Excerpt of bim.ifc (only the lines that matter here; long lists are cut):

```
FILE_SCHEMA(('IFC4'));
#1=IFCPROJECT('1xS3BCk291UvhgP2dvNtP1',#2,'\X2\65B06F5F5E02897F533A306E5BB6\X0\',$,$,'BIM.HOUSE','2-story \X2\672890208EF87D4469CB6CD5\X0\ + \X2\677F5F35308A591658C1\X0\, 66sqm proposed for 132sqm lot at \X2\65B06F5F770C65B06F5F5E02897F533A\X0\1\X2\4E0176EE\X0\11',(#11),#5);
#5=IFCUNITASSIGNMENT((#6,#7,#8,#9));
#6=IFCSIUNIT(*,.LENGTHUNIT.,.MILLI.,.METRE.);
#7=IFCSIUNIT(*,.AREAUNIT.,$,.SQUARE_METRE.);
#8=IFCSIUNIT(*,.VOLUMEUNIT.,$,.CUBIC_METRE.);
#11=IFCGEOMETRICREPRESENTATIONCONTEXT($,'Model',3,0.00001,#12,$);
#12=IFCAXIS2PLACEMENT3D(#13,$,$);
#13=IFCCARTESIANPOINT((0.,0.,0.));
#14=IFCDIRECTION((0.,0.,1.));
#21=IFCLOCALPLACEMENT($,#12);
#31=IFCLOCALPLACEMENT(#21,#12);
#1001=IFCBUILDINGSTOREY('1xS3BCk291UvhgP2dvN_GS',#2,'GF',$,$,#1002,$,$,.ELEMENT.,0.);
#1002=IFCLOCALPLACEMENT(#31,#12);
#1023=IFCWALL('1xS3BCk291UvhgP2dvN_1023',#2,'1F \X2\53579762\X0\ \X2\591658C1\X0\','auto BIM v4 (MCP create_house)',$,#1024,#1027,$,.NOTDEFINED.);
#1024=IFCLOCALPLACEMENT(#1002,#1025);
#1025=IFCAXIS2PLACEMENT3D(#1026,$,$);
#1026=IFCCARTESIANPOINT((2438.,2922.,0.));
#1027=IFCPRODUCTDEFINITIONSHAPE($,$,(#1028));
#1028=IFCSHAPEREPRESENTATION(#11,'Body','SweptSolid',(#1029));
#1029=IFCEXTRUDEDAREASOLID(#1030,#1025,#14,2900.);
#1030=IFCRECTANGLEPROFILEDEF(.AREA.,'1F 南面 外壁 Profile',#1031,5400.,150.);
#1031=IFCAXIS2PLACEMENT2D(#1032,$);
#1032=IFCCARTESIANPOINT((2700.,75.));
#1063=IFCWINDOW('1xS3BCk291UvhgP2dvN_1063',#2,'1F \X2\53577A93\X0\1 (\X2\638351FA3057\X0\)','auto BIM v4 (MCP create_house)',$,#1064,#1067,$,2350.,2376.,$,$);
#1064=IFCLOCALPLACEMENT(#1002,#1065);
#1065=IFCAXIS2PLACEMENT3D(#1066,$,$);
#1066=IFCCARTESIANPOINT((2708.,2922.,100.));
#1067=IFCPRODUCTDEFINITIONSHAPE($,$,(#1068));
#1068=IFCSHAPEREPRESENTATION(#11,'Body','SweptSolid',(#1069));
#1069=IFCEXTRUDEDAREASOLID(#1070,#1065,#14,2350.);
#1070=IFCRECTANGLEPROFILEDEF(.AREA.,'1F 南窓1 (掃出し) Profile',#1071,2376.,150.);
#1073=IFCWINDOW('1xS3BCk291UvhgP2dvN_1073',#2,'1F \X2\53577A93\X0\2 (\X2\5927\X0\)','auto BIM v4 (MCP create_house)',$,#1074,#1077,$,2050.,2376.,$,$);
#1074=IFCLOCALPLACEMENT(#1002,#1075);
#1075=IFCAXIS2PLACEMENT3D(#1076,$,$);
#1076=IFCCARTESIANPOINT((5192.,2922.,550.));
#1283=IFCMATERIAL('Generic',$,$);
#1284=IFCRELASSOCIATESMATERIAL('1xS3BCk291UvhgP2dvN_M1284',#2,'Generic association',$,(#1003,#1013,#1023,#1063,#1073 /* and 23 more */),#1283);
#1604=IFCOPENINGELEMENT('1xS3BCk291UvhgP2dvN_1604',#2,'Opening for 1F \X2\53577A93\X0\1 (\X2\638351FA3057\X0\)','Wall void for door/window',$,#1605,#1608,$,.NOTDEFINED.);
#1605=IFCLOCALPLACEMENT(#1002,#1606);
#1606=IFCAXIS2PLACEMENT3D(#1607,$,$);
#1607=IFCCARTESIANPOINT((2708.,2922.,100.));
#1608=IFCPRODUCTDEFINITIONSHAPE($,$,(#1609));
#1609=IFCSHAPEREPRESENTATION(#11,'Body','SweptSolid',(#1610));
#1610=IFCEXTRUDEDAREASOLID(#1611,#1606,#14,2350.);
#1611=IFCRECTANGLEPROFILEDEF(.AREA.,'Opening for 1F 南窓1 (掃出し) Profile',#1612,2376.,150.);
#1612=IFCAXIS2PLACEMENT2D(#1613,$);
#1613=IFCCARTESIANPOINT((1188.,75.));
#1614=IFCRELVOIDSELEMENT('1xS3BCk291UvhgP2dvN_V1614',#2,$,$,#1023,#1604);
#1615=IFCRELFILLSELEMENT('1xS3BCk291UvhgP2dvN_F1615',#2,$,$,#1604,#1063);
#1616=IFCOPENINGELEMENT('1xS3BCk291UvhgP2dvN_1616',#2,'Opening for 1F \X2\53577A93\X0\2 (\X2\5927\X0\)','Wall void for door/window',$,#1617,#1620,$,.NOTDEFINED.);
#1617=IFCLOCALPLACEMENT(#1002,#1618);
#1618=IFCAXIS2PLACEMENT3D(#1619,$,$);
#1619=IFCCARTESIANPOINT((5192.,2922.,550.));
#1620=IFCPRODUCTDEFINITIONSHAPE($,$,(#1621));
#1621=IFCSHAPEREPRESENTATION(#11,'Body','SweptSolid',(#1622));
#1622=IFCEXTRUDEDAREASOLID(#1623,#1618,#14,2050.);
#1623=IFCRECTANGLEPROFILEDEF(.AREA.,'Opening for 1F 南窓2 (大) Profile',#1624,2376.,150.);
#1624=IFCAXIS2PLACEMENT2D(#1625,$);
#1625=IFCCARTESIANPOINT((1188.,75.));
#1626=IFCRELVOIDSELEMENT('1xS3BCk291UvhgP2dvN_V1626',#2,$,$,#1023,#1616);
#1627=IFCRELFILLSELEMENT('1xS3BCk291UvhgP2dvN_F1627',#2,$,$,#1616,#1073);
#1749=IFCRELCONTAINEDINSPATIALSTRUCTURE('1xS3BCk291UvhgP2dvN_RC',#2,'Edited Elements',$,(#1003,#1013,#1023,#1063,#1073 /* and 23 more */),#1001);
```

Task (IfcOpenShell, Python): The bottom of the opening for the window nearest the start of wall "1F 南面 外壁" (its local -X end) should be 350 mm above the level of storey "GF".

```python
import numpy as np
import ifcopenshell
import ifcopenshell.api.geometry
import ifcopenshell.geom
import ifcopenshell.util.element
import ifcopenshell.util.placement
import ifcopenshell.util.shape
import ifcopenshell.util.unit

model = ifcopenshell.open("bim.ifc")
unit_scale = ifcopenshell.util.unit.calculate_unit_scale(model)

window = model.by_id(1063)
opening = window.FillsVoids[0].RelatingOpeningElement
storey = ifcopenshell.util.element.get_container(window, ifc_class="IfcBuildingStorey")
level = ifcopenshell.util.placement.get_local_placement(storey.ObjectPlacement)[2, 3]

# The opening's origin need not be at the sill, so measure its lowest point.
shape = ifcopenshell.geom.create_shape(ifcopenshell.geom.settings(), opening)
bottom = ifcopenshell.util.shape.get_shape_bottom_elevation(shape, shape.geometry) / unit_scale
dz = level + 0.35 / unit_scale - bottom

shift = np.array([0.0, 0.0, dz])
# The window is not placed relative to its opening, so move both.
for product in (opening, window):
    matrix = ifcopenshell.util.placement.get_local_placement(product.ObjectPlacement)
    matrix[:3, 3] += shift
    ifcopenshell.api.geometry.edit_object_placement(model, product=product, matrix=matrix, is_si=False)

print(f"moved by {dz * unit_scale:+.3f} m")

model.write("bim_updated.ifc")
```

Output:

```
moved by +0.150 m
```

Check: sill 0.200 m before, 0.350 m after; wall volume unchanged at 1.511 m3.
